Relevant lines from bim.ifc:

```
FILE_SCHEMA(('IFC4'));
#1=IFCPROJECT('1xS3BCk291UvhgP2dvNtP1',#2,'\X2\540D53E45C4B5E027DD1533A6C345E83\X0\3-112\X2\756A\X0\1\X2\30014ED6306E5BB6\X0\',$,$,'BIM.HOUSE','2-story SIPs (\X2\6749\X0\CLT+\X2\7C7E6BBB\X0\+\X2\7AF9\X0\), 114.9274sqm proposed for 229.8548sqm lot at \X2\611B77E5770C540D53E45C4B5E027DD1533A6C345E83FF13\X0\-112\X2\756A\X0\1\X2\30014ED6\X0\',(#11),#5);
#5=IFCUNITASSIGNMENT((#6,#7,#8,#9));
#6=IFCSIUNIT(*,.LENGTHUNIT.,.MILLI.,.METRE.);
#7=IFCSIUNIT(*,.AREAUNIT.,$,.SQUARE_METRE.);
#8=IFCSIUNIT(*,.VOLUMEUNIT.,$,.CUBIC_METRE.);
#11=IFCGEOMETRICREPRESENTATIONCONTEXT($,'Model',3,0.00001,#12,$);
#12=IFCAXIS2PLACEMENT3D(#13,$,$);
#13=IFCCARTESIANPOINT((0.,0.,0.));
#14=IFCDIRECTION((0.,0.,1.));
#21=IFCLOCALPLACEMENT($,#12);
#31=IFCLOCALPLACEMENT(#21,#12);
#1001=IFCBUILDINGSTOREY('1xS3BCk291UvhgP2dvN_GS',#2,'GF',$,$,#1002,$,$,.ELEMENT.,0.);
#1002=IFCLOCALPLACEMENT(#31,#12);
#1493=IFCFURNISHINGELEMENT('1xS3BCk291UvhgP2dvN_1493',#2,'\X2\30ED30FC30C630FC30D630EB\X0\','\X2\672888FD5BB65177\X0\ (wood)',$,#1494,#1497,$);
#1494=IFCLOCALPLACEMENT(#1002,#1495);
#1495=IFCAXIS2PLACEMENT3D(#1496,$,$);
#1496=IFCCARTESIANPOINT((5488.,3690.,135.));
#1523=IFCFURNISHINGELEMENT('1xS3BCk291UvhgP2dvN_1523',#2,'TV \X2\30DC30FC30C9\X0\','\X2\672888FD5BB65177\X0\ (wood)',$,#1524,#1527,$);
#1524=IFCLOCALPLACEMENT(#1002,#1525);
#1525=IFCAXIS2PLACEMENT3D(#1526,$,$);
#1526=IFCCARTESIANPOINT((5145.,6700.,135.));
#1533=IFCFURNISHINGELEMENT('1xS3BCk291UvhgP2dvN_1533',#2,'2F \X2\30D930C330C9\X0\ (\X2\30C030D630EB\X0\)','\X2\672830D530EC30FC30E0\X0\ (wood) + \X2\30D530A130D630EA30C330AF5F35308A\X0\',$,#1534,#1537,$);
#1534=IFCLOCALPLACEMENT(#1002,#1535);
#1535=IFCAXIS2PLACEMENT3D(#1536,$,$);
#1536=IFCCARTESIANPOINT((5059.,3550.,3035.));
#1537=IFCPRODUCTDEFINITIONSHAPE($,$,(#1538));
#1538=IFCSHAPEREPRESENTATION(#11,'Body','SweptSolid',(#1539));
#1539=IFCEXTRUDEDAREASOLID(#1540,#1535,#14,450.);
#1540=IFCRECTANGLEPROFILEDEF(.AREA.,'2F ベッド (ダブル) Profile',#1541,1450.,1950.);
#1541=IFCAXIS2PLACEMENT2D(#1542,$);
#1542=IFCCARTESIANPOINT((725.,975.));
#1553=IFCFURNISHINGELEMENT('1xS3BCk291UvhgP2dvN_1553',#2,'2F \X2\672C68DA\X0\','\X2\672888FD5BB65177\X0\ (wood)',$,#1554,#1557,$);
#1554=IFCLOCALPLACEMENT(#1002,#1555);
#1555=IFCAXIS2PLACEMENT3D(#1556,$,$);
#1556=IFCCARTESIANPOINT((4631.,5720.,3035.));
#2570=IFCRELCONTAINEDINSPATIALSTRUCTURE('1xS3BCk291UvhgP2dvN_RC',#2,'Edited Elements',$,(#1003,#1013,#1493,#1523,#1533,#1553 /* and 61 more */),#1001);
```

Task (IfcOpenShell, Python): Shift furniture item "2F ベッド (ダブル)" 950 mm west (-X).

```python
import ifcopenshell
import ifcopenshell.api.geometry
import ifcopenshell.util.placement

model = ifcopenshell.open("bim.ifc")

item = model.by_guid("1xS3BCk291UvhgP2dvN_1533")
matrix = ifcopenshell.util.placement.get_local_placement(item.ObjectPlacement)
matrix[0, 3] -= 950.0
ifcopenshell.api.geometry.edit_object_placement(model, product=item, matrix=matrix, is_si=False)

print(ifcopenshell.util.placement.get_local_placement(item.ObjectPlacement).round(3) + 0.0)

model.write("bim_rev.ifc")
```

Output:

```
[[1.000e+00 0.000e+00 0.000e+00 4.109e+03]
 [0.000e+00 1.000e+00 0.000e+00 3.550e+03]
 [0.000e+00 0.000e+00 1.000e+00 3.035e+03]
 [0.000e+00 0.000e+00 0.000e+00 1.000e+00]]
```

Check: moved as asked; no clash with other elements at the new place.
